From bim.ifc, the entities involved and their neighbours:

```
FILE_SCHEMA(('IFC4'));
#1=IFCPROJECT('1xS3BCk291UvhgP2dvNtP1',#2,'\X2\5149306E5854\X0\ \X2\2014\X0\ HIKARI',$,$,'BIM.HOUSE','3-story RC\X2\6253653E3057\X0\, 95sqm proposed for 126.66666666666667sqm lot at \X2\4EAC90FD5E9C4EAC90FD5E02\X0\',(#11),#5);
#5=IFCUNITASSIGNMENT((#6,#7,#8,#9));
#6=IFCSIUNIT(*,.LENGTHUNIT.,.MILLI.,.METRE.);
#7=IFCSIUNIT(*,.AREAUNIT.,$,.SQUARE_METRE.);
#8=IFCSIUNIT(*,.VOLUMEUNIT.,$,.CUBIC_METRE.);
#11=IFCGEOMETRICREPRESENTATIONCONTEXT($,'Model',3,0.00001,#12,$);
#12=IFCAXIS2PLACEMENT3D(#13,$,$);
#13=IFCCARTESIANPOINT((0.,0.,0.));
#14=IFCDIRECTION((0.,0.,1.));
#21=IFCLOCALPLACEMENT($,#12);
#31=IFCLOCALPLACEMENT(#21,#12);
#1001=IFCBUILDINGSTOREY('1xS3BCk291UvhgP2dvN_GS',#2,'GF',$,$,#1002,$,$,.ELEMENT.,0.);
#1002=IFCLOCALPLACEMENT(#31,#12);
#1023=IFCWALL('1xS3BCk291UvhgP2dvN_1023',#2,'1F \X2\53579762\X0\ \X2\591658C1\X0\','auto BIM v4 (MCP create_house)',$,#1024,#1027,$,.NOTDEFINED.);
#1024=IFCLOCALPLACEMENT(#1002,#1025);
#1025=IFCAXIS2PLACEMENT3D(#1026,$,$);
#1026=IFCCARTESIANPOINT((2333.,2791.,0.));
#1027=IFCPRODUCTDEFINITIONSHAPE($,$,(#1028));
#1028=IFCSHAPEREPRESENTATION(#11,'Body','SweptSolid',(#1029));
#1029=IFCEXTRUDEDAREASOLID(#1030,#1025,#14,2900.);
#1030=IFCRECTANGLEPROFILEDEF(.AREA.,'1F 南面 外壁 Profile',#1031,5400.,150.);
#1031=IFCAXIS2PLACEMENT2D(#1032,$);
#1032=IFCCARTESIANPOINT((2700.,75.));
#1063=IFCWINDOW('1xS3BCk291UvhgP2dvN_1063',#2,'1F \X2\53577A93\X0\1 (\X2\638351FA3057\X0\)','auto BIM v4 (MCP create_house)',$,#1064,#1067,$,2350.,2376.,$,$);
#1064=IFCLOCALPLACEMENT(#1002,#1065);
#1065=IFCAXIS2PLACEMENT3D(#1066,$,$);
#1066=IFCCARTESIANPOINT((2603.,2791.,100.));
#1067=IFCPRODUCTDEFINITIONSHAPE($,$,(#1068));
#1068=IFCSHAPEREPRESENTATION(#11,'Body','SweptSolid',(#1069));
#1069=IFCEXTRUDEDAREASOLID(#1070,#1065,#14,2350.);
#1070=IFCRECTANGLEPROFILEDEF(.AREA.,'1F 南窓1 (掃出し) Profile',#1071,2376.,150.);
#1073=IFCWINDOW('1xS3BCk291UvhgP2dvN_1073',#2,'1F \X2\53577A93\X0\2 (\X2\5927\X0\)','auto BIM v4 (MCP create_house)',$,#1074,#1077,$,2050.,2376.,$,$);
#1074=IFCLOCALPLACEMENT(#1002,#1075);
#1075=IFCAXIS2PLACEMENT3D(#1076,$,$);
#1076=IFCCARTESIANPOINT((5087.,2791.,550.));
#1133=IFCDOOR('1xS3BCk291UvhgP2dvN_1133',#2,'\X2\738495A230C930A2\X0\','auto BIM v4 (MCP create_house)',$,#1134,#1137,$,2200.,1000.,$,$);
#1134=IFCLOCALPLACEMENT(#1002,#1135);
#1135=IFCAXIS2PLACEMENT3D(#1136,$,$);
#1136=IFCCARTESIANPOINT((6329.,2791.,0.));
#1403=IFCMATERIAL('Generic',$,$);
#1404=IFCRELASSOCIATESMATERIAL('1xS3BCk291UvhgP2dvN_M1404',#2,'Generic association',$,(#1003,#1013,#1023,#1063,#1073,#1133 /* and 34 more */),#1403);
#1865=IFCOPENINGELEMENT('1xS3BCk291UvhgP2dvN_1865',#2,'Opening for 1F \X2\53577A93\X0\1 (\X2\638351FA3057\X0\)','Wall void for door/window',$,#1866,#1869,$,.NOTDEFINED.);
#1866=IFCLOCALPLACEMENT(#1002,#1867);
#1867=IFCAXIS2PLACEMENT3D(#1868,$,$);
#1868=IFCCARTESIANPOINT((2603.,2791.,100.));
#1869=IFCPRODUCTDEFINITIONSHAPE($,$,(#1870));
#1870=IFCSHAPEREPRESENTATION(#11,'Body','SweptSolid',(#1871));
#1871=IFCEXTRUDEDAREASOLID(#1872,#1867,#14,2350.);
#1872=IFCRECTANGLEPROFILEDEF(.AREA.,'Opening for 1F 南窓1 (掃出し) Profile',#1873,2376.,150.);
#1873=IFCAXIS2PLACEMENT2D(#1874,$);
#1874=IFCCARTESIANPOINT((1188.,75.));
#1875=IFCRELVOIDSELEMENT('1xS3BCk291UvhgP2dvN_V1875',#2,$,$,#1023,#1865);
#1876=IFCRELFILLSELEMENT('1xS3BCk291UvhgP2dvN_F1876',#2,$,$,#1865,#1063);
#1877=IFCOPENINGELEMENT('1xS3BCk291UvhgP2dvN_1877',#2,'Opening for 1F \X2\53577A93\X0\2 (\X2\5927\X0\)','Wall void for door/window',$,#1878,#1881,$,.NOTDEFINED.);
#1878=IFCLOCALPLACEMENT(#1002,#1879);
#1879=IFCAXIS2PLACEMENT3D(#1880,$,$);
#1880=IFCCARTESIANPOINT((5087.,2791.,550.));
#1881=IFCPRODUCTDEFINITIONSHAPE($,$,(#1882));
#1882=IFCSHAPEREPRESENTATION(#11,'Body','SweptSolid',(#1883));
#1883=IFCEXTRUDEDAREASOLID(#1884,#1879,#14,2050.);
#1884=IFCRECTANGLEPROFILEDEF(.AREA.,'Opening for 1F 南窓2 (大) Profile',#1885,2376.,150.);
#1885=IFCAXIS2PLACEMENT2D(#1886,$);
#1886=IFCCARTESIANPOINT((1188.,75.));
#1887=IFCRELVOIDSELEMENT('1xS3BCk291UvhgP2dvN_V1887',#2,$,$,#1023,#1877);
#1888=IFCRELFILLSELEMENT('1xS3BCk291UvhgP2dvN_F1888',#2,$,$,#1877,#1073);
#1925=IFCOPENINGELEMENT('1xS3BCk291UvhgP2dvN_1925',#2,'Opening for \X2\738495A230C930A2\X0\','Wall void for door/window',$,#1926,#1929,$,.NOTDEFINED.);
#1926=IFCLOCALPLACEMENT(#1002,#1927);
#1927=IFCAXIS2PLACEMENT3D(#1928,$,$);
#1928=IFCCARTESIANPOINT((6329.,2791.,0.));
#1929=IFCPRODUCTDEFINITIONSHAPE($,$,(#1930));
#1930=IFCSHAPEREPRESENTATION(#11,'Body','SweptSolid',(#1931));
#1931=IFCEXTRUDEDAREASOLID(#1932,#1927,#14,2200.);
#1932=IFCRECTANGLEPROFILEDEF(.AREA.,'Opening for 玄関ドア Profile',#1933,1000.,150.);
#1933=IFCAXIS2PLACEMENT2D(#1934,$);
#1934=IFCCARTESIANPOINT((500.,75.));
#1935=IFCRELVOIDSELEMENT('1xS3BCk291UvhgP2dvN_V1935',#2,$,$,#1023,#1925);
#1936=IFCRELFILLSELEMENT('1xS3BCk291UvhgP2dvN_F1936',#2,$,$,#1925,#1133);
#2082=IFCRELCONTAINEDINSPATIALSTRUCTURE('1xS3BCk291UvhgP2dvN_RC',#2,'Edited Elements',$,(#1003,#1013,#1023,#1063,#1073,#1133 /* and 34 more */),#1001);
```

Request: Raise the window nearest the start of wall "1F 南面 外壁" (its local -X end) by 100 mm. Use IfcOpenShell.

```python
import numpy as np
import ifcopenshell
import ifcopenshell.api.geometry
import ifcopenshell.util.placement
import ifcopenshell.util.unit

model = ifcopenshell.open("bim.ifc")
unit_scale = ifcopenshell.util.unit.calculate_unit_scale(model)

window = model.by_id(1063)
opening = window.FillsVoids[0].RelatingOpeningElement
dz = 0.1 / unit_scale

shift = np.array([0.0, 0.0, dz])
# The window is not placed relative to its opening, so move both.
for product in (opening, window):
    matrix = ifcopenshell.util.placement.get_local_placement(product.ObjectPlacement)
    matrix[:3, 3] += shift
    ifcopenshell.api.geometry.edit_object_placement(model, product=product, matrix=matrix, is_si=False)

print(f"moved by {dz * unit_scale:+.3f} m")

model.write("bim_edited.ifc")
```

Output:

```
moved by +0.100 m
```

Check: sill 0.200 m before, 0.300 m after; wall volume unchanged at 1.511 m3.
